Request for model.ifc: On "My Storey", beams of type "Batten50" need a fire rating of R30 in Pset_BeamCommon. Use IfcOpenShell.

First a look at what the model holds.

```python
import ifcopenshell
import ifcopenshell.util.element

model = ifcopenshell.open("model.ifc")
print(model.schema)
storey = next(s for s in model.by_type("IfcBuildingStorey") if s.Name == "My Storey")
beams = [e for e in ifcopenshell.util.element.get_decomposition(storey) if e.is_a("IfcBeam")]
seen = {}
for e in beams:
    element_type = ifcopenshell.util.element.get_type(e)
    key = (element_type.Name if element_type != e and element_type else None, ifcopenshell.util.element.get_pset(e, "Pset_BeamCommon", "FireRating"))
    seen[key] = seen.get(key, 0) + 1
for (name, value), count in sorted(seen.items(), key=str):
    print(count, "x", name, "|", value)
```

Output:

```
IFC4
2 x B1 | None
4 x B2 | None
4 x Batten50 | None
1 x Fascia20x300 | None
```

```python
import ifcopenshell
import ifcopenshell.api.pset
import ifcopenshell.util.element

model = ifcopenshell.open("model.ifc")

storey = next(s for s in model.by_type("IfcBuildingStorey") if s.Name == "My Storey")
beams = [e for e in ifcopenshell.util.element.get_decomposition(storey) if e.is_a("IfcBeam")]

count = 0
for e in beams:
    element_type = ifcopenshell.util.element.get_type(e)
    if element_type in (None, e) or element_type.Name != "Batten50":
        continue
    # add_pset returns the element's existing set when there is one.
    pset = ifcopenshell.api.pset.add_pset(model, product=e, name="Pset_BeamCommon")
    ifcopenshell.api.pset.edit_pset(model, pset=pset, properties={"FireRating": "R30"})
    count += 1

print(count, "beams updated")

model.write("model-out.ifc")
```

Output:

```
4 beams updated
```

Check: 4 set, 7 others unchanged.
